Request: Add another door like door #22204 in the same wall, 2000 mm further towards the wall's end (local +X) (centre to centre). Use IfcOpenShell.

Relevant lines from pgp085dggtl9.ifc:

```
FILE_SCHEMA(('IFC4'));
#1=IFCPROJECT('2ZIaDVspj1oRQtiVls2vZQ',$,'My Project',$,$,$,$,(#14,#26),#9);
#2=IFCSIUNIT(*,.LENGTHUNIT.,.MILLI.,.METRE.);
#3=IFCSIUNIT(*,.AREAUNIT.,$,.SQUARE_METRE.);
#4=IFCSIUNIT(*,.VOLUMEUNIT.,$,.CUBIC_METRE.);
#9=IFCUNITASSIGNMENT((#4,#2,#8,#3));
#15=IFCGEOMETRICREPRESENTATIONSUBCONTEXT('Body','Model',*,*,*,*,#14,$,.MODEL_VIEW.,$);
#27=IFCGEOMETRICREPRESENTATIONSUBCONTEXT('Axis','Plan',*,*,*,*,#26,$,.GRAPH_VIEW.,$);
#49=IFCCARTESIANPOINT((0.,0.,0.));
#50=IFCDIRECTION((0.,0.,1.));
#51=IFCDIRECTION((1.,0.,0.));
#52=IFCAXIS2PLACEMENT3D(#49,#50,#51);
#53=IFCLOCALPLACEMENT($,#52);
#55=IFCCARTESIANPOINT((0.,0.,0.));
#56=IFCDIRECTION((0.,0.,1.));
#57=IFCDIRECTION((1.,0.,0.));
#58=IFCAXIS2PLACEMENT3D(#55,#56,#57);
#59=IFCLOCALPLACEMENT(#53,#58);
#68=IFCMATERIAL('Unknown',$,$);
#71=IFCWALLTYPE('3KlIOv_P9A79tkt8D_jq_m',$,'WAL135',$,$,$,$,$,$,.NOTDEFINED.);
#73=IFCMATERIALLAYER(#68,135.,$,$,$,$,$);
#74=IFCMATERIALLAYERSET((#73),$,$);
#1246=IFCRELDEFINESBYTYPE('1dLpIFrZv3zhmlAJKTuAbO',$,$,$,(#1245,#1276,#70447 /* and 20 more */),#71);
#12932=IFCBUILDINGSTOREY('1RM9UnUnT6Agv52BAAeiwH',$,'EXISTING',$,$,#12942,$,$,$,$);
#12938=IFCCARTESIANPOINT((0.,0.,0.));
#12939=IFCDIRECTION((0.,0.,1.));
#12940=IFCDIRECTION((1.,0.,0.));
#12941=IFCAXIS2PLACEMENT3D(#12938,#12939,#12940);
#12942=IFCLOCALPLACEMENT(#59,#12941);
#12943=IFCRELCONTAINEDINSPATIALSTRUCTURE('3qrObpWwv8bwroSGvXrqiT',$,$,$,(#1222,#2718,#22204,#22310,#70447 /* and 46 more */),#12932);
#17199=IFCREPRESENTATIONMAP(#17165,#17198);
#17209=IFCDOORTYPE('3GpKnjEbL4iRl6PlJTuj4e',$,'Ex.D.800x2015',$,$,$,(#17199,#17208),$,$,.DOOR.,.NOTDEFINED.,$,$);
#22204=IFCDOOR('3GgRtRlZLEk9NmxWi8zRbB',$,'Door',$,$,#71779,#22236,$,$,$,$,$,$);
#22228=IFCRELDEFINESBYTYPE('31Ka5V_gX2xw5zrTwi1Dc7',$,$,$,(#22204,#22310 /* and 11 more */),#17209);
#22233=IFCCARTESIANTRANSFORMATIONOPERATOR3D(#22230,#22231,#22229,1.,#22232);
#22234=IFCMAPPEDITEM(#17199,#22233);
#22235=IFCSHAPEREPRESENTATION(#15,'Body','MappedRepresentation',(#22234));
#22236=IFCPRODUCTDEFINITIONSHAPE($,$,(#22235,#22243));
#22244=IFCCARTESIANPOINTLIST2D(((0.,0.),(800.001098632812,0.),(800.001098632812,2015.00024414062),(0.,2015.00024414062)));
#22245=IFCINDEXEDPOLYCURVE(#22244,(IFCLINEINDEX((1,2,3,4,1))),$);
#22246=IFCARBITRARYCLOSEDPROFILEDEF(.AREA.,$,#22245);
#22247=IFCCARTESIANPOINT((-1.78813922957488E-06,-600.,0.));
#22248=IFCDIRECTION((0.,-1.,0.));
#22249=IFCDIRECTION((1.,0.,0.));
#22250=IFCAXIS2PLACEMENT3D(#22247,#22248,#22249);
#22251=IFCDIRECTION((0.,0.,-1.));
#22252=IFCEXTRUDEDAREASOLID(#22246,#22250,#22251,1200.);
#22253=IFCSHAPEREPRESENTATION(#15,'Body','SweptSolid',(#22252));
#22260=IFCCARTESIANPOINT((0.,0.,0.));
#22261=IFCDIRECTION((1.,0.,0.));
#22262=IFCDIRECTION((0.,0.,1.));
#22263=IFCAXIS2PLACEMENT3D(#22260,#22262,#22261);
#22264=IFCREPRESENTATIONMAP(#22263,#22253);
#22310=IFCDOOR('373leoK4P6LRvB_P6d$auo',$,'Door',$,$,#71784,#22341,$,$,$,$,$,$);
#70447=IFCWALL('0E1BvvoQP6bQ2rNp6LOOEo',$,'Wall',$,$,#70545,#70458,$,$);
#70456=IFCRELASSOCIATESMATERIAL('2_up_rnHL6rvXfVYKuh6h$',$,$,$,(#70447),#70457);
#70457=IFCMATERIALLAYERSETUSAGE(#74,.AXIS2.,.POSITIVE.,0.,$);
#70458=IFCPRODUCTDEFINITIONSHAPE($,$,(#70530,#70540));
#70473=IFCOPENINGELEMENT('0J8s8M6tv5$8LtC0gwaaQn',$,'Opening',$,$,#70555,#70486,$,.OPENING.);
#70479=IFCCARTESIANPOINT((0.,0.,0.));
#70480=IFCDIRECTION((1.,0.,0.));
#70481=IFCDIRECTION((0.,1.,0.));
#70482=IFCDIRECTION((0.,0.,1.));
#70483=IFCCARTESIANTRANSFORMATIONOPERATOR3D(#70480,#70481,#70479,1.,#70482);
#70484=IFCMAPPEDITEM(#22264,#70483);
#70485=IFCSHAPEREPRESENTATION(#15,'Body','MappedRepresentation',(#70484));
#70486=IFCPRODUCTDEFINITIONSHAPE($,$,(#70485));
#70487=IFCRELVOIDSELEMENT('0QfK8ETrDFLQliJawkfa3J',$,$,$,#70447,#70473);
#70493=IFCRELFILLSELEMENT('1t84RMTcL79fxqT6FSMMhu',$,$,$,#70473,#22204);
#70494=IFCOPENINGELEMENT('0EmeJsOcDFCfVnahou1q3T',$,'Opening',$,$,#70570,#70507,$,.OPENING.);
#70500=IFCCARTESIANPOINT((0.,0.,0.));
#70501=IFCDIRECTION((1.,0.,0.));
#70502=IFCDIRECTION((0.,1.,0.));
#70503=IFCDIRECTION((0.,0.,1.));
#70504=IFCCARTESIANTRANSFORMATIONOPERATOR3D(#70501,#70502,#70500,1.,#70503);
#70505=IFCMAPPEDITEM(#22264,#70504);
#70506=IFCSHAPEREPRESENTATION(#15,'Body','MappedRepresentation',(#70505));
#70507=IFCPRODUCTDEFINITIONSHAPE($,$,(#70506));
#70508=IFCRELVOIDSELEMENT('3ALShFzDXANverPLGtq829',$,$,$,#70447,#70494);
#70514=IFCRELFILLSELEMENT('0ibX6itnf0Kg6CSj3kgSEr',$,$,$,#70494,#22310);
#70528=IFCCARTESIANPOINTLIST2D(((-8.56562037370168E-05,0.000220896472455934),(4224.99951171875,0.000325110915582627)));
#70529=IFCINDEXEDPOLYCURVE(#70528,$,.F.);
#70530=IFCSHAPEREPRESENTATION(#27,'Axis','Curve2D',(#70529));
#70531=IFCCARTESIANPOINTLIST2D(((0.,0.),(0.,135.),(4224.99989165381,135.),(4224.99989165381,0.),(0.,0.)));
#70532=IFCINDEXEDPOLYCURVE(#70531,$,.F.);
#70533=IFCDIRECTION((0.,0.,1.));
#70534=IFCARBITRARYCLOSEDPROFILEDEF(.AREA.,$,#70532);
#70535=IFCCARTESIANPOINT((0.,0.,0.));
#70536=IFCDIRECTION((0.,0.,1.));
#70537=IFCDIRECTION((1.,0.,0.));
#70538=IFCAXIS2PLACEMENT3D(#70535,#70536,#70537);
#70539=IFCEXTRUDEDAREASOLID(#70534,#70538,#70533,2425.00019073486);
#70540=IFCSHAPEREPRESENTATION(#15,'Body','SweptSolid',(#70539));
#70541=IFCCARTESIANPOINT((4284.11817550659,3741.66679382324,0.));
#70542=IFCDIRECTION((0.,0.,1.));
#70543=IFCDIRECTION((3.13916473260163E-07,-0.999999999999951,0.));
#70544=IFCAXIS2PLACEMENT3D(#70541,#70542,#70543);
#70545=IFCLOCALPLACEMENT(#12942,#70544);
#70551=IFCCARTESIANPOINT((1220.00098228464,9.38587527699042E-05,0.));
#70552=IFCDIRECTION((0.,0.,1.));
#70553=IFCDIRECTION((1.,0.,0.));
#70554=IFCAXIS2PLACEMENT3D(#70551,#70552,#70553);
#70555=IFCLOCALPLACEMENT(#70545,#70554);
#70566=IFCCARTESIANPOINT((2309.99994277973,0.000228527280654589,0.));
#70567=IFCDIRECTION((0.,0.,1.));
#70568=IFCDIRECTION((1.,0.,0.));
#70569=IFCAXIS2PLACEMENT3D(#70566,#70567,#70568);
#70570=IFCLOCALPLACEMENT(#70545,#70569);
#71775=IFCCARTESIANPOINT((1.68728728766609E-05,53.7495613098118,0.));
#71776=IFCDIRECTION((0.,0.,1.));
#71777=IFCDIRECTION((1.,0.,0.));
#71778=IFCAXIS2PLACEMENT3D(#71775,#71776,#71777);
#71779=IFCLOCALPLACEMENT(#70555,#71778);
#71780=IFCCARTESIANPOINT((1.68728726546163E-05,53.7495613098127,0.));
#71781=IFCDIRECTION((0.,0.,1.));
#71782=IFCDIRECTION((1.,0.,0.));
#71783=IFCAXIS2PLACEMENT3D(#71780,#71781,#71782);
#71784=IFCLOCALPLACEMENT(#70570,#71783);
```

```python
import ifcopenshell
import ifcopenshell.api.feature
import ifcopenshell.api.geometry
import ifcopenshell.api.root
import ifcopenshell.geom
import ifcopenshell.util.element
import ifcopenshell.util.placement
import ifcopenshell.util.shape
import ifcopenshell.util.unit

model = ifcopenshell.open("pgp085dggtl9.ifc")
unit_scale = ifcopenshell.util.unit.calculate_unit_scale(model)
settings = ifcopenshell.geom.settings()


def volume(element):
    """Net volume in cubic metres, openings subtracted."""
    shape = ifcopenshell.geom.create_shape(settings, element)
    return ifcopenshell.util.shape.get_volume(shape.geometry)


door = model.by_guid("3GgRtRlZLEk9NmxWi8zRbB")
opening = door.FillsVoids[0].RelatingOpeningElement
wall = opening.VoidsElements[0].RelatingBuildingElement
before = volume(wall)
shift = ifcopenshell.util.placement.get_local_placement(wall.ObjectPlacement)[:3, 0] * 2 / unit_scale

# copy_class copies the void relationship, type, container and properties, but no geometry.
new_opening = ifcopenshell.api.root.copy_class(model, product=opening)
new_opening.Representation = ifcopenshell.util.element.copy_deep(
    model, opening.Representation, exclude=["IfcGeometricRepresentationContext", "IfcRepresentationMap"]
)
new_door = ifcopenshell.api.root.copy_class(model, product=door)
new_door.Representation = ifcopenshell.util.element.copy_deep(
    model, door.Representation, exclude=["IfcGeometricRepresentationContext", "IfcRepresentationMap"]
)
ifcopenshell.api.feature.add_filling(model, opening=new_opening, element=new_door)

for old, new in ((opening, new_opening), (door, new_door)):
    matrix = ifcopenshell.util.placement.get_local_placement(old.ObjectPlacement)
    matrix[:3, 3] += shift
    ifcopenshell.api.geometry.edit_object_placement(model, product=new, matrix=matrix, is_si=False)

after = volume(wall)

print(f"wall volume {before:.3f} -> {after:.3f} m3")

model.write("pgp085dggtl9_updated.ifc")
```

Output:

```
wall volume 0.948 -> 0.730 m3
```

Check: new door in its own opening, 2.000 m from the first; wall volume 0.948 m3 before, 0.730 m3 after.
